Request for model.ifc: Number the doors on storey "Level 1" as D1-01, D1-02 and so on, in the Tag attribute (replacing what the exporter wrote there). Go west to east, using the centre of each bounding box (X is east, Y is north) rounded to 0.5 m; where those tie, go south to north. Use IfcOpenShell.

First a look at what the model holds.

```python
import ifcopenshell
import ifcopenshell.util.element
import ifcopenshell.util.placement

model = ifcopenshell.open("model.ifc")
print(model.schema)
storey = next(s for s in model.by_type("IfcBuildingStorey") if s.Name == "Level 1")
doors = [e for e in ifcopenshell.util.element.get_decomposition(storey) if e.is_a("IfcDoor")]
for e in sorted(doors, key=lambda e: e.id()):
    origin = ifcopenshell.util.placement.get_local_placement(e.ObjectPlacement)[:3, 3]
    print(e.id(), e.Tag, e.Name, origin.round(2) + 0.0, sep=" | ")
```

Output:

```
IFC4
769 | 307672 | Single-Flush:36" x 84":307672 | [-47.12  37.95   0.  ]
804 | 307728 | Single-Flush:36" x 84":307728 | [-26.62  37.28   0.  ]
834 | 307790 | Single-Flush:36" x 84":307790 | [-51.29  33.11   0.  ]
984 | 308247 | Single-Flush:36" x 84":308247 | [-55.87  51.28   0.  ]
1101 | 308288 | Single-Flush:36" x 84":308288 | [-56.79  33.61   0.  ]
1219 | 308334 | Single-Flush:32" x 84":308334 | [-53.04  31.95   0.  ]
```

```python
import ifcopenshell
import ifcopenshell.geom
import ifcopenshell.util.element
import ifcopenshell.util.shape

model = ifcopenshell.open("model.ifc")
settings = ifcopenshell.geom.settings()
settings.set("use-world-coords", True)


def centre(element):
    shape = ifcopenshell.geom.create_shape(settings, element)
    return ifcopenshell.util.shape.get_bbox_centroid(shape.geometry)


storey = next(s for s in model.by_type("IfcBuildingStorey") if s.Name == "Level 1")
doors = [e for e in ifcopenshell.util.element.get_decomposition(storey) if e.is_a("IfcDoor")]

# Insertion points can sit at a corner or the storey origin, so sort by the geometry (in metres).
centres = {e: centre(e) for e in doors}
doors.sort(key=lambda e: (round(centres[e][0] / 0.5), centres[e][1]))

for i, e in enumerate(doors, start=1):
    number = f"D1-{i:02d}"
    e.Tag = number
    print(e.id(), number)

model.write("model_edited.ifc")
```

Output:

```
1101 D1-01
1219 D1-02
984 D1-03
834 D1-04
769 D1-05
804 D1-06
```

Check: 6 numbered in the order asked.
